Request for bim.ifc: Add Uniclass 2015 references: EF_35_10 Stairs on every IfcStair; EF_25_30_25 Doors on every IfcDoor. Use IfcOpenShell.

First a look at what the model holds.

```python
import ifcopenshell

model = ifcopenshell.open("bim.ifc")
print(model.schema)
print("classifications:", [c.Name for c in model.by_type("IfcClassification")])
for ifc_class in ("IfcDoor", "IfcRoof", "IfcStair", "IfcWall", "IfcWindow"):
    print(ifc_class, len(model.by_type(ifc_class)))
```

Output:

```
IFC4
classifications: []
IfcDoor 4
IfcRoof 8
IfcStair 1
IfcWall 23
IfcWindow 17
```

```python
import ifcopenshell
import ifcopenshell.api.classification

model = ifcopenshell.open("bim.ifc")

system = ifcopenshell.api.classification.add_classification(model, classification="Uniclass 2015")

codes = {
    "IfcStair": ("EF_35_10", "Stairs"),
    "IfcDoor": ("EF_25_30_25", "Doors"),
}
for ifc_class, (code, name) in codes.items():
    products = model.by_type(ifc_class)
    ifcopenshell.api.classification.add_reference(
        model, products=products, classification=system, identification=code, name=name
    )
    print(code, len(products))

model.write("bim_edited.ifc")
```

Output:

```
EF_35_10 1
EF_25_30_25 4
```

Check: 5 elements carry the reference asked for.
